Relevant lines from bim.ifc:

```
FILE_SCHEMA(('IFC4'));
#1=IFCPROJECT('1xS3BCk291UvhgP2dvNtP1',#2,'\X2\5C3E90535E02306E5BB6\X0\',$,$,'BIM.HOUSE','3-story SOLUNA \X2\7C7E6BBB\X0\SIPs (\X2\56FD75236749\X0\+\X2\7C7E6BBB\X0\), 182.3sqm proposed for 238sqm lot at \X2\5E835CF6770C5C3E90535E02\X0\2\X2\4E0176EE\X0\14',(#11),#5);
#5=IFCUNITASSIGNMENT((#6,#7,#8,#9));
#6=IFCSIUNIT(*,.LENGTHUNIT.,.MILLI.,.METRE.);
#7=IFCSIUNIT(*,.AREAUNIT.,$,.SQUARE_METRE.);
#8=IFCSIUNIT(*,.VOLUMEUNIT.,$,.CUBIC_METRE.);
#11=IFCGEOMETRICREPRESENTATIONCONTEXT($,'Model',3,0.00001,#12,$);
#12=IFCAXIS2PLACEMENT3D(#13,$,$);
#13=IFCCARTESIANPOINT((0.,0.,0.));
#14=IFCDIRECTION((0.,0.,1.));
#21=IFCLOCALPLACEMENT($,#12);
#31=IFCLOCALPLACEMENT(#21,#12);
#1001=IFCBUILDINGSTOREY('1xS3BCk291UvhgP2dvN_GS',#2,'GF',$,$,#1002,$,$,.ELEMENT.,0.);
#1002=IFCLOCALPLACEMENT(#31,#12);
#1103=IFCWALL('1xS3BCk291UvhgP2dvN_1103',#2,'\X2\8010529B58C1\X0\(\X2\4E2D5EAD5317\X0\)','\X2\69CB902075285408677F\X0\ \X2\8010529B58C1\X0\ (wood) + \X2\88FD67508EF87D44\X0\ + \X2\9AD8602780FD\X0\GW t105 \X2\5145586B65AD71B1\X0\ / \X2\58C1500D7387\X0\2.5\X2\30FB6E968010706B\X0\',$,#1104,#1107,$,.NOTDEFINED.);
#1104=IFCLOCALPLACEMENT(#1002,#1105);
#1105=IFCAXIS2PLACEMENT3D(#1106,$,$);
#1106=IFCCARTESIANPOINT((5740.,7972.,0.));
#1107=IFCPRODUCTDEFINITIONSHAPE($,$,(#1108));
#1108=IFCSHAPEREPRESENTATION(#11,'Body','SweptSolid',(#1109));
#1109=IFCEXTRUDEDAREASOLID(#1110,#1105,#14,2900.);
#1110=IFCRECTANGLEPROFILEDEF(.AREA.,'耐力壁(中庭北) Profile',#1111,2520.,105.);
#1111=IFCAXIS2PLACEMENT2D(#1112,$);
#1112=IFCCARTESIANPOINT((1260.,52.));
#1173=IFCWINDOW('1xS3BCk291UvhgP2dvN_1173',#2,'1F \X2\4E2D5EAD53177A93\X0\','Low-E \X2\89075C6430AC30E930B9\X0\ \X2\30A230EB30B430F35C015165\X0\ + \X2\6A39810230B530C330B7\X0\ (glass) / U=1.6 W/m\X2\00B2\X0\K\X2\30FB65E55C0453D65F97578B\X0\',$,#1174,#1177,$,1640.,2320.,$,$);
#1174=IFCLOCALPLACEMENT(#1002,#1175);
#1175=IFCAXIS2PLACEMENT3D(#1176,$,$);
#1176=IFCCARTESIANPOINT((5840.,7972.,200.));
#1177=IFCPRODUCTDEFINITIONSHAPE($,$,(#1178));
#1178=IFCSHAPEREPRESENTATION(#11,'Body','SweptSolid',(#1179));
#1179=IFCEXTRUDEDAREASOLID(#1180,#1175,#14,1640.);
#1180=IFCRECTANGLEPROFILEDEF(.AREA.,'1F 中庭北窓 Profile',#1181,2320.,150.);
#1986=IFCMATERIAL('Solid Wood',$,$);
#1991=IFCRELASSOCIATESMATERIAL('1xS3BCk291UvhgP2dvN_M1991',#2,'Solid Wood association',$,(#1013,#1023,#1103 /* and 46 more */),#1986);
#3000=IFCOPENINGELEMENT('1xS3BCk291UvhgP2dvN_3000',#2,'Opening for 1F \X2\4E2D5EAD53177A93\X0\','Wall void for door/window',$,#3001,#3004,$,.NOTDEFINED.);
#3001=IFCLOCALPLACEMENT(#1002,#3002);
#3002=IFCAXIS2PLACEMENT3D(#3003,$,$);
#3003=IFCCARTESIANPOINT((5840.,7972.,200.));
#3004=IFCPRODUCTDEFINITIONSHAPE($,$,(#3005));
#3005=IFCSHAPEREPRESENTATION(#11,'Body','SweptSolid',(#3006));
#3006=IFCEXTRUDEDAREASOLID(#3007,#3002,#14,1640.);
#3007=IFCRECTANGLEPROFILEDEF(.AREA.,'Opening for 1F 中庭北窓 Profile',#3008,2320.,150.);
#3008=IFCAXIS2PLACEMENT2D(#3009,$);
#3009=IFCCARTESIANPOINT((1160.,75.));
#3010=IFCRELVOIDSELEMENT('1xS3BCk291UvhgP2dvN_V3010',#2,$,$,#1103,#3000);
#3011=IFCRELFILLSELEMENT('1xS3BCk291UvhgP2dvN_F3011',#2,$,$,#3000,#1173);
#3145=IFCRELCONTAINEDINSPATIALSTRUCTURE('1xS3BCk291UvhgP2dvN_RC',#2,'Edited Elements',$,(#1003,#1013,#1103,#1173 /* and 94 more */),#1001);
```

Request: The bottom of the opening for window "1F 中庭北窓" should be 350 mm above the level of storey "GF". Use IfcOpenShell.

```python
import numpy as np
import ifcopenshell
import ifcopenshell.api.geometry
import ifcopenshell.geom
import ifcopenshell.util.element
import ifcopenshell.util.placement
import ifcopenshell.util.shape
import ifcopenshell.util.unit

model = ifcopenshell.open("bim.ifc")
unit_scale = ifcopenshell.util.unit.calculate_unit_scale(model)

window = model.by_guid("1xS3BCk291UvhgP2dvN_1173")
opening = window.FillsVoids[0].RelatingOpeningElement
storey = ifcopenshell.util.element.get_container(window, ifc_class="IfcBuildingStorey")
level = ifcopenshell.util.placement.get_local_placement(storey.ObjectPlacement)[2, 3]

# The opening's origin need not be at the sill, so measure its lowest point.
shape = ifcopenshell.geom.create_shape(ifcopenshell.geom.settings(), opening)
bottom = ifcopenshell.util.shape.get_shape_bottom_elevation(shape, shape.geometry) / unit_scale
dz = level + 0.35 / unit_scale - bottom

shift = np.array([0.0, 0.0, dz])
# The window is not placed relative to its opening, so move both.
for product in (opening, window):
    matrix = ifcopenshell.util.placement.get_local_placement(product.ObjectPlacement)
    matrix[:3, 3] += shift
    ifcopenshell.api.geometry.edit_object_placement(model, product=product, matrix=matrix, is_si=False)

print(f"moved by {dz * unit_scale:+.3f} m")

model.write("bim_updated.ifc")
```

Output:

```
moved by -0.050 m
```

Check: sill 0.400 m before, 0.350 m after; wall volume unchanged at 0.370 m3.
